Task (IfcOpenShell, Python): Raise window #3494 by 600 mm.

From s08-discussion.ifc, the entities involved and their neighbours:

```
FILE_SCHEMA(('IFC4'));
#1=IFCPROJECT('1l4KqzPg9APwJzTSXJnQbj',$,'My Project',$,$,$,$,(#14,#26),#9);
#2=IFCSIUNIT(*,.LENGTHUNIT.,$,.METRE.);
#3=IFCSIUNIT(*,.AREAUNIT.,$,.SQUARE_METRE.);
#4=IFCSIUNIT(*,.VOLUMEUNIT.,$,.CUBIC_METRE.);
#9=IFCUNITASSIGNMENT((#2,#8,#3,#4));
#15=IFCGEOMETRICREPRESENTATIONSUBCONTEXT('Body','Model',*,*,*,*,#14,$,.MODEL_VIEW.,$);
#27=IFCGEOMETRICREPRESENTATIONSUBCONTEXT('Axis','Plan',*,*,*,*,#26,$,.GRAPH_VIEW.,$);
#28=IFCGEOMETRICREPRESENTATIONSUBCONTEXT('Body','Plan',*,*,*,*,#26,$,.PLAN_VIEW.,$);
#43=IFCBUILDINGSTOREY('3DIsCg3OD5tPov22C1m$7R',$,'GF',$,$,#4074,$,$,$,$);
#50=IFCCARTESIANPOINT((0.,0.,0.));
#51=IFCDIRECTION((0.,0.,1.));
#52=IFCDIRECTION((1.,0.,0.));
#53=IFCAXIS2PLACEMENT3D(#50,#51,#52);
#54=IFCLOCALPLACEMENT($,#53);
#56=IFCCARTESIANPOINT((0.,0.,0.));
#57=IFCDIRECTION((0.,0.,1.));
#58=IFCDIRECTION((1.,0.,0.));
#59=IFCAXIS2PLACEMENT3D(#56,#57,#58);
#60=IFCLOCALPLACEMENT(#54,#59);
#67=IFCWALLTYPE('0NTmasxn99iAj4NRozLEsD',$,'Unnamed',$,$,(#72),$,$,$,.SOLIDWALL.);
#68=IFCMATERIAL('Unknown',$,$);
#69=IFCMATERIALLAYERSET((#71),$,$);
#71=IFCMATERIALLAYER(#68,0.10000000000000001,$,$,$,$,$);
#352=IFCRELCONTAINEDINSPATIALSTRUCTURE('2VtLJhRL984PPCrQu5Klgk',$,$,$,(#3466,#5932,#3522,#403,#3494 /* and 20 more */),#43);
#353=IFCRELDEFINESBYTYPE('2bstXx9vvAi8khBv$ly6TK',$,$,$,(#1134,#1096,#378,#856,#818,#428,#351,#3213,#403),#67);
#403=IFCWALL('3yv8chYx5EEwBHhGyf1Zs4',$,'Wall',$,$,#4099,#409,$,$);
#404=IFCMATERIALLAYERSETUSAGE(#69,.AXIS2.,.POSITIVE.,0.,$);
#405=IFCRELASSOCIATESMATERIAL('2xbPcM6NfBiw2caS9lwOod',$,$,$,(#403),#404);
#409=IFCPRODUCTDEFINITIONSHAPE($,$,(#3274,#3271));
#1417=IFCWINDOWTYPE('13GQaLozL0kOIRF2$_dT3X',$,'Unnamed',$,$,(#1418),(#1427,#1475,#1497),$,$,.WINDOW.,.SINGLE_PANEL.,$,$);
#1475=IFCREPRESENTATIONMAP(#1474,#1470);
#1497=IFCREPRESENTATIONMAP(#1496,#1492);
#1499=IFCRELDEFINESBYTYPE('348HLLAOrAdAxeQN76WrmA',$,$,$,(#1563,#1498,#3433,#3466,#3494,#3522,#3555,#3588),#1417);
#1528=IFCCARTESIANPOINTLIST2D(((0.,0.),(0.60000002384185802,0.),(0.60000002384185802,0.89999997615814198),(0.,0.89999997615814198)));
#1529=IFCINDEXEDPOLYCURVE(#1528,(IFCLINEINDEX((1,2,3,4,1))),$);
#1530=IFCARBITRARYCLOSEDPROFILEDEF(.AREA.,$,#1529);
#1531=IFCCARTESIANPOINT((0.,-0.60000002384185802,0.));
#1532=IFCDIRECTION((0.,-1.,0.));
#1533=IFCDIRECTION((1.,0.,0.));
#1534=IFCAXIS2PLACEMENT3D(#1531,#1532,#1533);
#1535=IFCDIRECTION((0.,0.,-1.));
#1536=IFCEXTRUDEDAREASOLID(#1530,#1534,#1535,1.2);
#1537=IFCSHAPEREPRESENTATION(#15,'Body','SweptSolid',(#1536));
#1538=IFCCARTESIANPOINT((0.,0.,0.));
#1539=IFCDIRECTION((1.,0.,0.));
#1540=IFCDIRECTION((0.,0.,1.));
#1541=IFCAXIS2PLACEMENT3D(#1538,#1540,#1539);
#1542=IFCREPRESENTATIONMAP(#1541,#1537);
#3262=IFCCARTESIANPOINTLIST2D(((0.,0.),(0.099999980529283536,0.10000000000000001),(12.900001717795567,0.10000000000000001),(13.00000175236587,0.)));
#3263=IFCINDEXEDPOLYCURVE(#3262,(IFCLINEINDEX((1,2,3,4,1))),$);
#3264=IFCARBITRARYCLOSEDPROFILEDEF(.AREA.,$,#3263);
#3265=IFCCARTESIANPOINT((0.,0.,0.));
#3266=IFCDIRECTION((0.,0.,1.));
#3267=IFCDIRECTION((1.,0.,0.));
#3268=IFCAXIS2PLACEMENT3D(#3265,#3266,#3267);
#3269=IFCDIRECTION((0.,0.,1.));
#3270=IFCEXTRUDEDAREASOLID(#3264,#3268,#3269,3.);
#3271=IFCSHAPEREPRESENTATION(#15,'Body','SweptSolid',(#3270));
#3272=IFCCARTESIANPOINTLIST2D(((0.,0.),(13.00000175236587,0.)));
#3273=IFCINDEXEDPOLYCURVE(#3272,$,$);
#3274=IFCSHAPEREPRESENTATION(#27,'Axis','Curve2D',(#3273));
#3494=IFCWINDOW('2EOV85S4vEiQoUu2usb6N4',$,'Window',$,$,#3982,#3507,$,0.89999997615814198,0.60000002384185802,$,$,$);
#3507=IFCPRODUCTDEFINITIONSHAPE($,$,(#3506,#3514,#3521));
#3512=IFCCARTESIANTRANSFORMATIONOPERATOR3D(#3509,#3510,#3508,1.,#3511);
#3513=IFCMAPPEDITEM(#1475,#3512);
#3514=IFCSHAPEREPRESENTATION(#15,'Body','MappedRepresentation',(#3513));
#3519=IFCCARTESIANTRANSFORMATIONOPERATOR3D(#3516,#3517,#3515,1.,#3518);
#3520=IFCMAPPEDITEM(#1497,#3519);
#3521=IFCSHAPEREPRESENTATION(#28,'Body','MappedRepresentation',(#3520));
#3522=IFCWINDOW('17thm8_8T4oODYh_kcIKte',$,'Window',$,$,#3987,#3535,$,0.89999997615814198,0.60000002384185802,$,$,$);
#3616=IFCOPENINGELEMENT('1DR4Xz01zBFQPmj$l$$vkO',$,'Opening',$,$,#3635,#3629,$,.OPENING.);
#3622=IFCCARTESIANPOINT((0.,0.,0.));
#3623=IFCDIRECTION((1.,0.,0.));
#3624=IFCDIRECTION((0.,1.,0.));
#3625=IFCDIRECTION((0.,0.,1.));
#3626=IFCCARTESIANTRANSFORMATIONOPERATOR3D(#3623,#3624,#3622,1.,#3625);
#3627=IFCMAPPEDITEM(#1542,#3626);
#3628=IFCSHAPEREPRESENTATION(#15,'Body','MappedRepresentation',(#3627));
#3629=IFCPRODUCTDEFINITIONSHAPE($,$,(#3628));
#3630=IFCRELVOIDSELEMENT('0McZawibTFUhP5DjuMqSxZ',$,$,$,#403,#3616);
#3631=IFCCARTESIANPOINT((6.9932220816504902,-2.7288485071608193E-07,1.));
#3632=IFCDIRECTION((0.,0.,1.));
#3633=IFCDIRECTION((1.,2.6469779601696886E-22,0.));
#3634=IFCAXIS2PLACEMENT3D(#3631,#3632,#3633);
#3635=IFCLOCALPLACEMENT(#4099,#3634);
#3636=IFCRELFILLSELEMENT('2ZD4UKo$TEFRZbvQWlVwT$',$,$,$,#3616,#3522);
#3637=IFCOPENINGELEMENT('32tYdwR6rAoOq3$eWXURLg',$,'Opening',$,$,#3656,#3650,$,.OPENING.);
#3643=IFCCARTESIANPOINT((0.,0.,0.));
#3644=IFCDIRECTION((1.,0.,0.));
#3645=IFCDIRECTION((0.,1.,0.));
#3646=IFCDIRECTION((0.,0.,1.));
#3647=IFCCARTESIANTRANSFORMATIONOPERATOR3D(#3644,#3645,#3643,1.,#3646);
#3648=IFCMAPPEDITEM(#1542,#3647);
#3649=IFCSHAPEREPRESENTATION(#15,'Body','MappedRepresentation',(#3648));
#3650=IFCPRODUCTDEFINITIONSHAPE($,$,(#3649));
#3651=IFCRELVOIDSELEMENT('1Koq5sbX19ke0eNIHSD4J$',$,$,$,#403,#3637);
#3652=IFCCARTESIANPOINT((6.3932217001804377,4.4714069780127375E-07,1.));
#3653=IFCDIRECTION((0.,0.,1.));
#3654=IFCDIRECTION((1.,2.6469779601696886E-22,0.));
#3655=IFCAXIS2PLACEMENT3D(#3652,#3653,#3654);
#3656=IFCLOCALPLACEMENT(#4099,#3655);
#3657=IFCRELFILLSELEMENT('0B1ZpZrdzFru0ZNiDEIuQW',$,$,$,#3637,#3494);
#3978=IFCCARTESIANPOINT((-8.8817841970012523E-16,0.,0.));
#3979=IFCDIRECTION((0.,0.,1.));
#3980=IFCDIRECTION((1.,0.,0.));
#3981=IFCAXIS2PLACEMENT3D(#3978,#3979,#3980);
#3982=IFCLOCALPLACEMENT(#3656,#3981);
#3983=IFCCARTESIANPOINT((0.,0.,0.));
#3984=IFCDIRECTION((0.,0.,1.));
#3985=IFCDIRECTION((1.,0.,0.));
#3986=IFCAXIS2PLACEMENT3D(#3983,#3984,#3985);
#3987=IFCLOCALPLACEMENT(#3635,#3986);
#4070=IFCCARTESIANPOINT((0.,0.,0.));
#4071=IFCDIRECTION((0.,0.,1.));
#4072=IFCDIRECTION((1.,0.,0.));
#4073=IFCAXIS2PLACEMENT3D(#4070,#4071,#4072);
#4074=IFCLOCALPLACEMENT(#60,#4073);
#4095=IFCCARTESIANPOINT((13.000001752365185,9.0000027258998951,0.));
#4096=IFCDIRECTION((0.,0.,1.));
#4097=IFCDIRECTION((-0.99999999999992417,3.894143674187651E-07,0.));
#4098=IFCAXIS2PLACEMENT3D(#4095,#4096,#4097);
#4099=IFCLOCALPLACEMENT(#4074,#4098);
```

```python
import numpy as np
import ifcopenshell
import ifcopenshell.api.geometry
import ifcopenshell.util.placement
import ifcopenshell.util.unit

model = ifcopenshell.open("s08-discussion.ifc")
unit_scale = ifcopenshell.util.unit.calculate_unit_scale(model)

window = model.by_id(3494)
opening = window.FillsVoids[0].RelatingOpeningElement
dz = 0.6 / unit_scale

shift = np.array([0.0, 0.0, dz])
# The window is placed relative to its opening, so it follows when the opening moves.
matrix = ifcopenshell.util.placement.get_local_placement(opening.ObjectPlacement)
matrix[:3, 3] += shift
ifcopenshell.api.geometry.edit_object_placement(
    model, product=opening, matrix=matrix, is_si=False, should_transform_children=True
)

print(f"moved by {dz * unit_scale:+.3f} m")

model.write("s08-discussion_v2.ifc")
```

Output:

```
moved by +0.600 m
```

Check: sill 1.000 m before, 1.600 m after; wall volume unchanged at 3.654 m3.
